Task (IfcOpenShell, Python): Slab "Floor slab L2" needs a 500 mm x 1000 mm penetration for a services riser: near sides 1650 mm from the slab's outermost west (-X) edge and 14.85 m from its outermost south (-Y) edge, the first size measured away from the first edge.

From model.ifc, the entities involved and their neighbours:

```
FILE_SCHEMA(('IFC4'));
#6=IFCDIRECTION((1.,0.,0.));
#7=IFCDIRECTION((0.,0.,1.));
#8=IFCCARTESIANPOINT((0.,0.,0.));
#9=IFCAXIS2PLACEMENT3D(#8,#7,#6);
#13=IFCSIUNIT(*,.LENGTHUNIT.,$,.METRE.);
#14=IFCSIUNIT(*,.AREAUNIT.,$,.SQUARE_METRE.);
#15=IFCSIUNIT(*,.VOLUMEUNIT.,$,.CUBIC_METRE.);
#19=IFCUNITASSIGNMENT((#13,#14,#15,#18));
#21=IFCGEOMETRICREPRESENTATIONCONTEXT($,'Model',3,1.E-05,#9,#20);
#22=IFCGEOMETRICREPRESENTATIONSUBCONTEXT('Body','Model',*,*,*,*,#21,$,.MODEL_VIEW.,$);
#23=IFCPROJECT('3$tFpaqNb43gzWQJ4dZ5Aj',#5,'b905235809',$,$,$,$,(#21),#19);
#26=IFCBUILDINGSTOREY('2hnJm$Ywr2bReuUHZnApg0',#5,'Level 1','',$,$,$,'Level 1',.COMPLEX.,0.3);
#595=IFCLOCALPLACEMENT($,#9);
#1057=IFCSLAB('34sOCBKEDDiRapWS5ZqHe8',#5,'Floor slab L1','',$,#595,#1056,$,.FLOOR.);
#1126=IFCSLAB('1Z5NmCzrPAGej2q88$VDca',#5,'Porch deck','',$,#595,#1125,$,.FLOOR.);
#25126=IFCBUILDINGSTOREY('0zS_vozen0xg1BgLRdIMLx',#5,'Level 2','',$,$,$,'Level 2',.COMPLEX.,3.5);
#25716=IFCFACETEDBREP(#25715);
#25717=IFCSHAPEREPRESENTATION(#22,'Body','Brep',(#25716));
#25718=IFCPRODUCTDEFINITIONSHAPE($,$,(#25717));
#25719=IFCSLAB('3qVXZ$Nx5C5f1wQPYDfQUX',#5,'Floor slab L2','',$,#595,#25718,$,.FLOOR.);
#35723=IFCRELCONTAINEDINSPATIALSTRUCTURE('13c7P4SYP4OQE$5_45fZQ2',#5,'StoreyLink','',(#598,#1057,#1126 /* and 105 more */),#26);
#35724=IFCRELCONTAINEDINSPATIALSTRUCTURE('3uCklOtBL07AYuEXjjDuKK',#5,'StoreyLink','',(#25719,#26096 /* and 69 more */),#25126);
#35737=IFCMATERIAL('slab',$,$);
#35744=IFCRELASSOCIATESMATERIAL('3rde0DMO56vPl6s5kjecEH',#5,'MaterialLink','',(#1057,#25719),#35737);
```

```python
import numpy as np
import ifcopenshell
import ifcopenshell.api.feature
import ifcopenshell.api.geometry
import ifcopenshell.api.root
import ifcopenshell.geom
import ifcopenshell.util.placement
import ifcopenshell.util.representation
import ifcopenshell.util.shape
import ifcopenshell.util.unit

model = ifcopenshell.open("model.ifc")
unit_scale = ifcopenshell.util.unit.calculate_unit_scale(model)
settings = ifcopenshell.geom.settings()


def volume(element):
    """Net volume in cubic metres, openings subtracted."""
    shape = ifcopenshell.geom.create_shape(settings, element)
    return ifcopenshell.util.shape.get_volume(shape.geometry)


slab = model.by_guid("3qVXZ$Nx5C5f1wQPYDfQUX")
before = volume(slab)

# Extent in the slab's own axes, in metres. The edges named are its -X and -Y sides.
slab_shape = ifcopenshell.geom.create_shape(settings, slab)
vertices = ifcopenshell.util.shape.get_vertices(slab_shape.geometry)
x_min, y_min, bottom = vertices.min(axis=0)
top = vertices[:, 2].max()

opening = ifcopenshell.api.root.create_entity(model, ifc_class="IfcOpeningElement", name="Services riser opening", predefined_type="OPENING")
context = ifcopenshell.util.representation.get_context(model, "Model", "Body", "MODEL_VIEW")
width, depth = 0.5, 1
outline = [(0.0, 0.0), (width, 0.0), (width, depth), (0.0, depth), (0.0, 0.0)]
# Overshoot both faces by 50 mm so the cut is clean.
shape = ifcopenshell.api.geometry.add_slab_representation(
    model, context=context, depth=top - bottom + 0.1, polyline=outline
)
ifcopenshell.api.geometry.assign_representation(model, product=opening, representation=shape)

matrix = ifcopenshell.util.placement.get_local_placement(slab.ObjectPlacement)
matrix[:, 3] = matrix @ np.append(np.array([x_min + 1.65, y_min + 14.85, bottom - 0.05]) / unit_scale, 1.0)
ifcopenshell.api.geometry.edit_object_placement(model, product=opening, matrix=matrix, is_si=False)
ifcopenshell.api.feature.add_feature(model, feature=opening, element=slab)

after = volume(slab)

print(f"slab volume {before:.3f} -> {after:.3f} m3")

model.write("model_v2.ifc")
```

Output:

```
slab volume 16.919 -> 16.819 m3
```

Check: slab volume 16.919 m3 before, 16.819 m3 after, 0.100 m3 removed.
